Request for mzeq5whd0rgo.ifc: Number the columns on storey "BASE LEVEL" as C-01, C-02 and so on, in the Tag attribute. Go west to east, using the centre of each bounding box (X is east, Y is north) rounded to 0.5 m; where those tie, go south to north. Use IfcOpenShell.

First a look at what the model holds.

```python
import ifcopenshell
import ifcopenshell.util.element
import ifcopenshell.util.placement

model = ifcopenshell.open("mzeq5whd0rgo.ifc")
print(model.schema)
storey = next(s for s in model.by_type("IfcBuildingStorey") if s.Name == "BASE LEVEL")
columns = [e for e in ifcopenshell.util.element.get_decomposition(storey) if e.is_a("IfcColumn")]
for e in sorted(columns, key=lambda e: e.id()):
    origin = ifcopenshell.util.placement.get_local_placement(e.ObjectPlacement)[:3, 3]
    print(e.id(), e.Tag, e.Name, origin.round(2) + 0.0, sep=" | ")
```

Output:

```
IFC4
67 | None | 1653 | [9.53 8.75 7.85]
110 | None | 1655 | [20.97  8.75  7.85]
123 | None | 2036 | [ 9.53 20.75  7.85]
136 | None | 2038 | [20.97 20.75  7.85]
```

```python
import ifcopenshell
import ifcopenshell.geom
import ifcopenshell.util.element
import ifcopenshell.util.shape

model = ifcopenshell.open("mzeq5whd0rgo.ifc")
settings = ifcopenshell.geom.settings()
settings.set("use-world-coords", True)


def centre(element):
    shape = ifcopenshell.geom.create_shape(settings, element)
    return ifcopenshell.util.shape.get_bbox_centroid(shape.geometry)


storey = next(s for s in model.by_type("IfcBuildingStorey") if s.Name == "BASE LEVEL")
columns = [e for e in ifcopenshell.util.element.get_decomposition(storey) if e.is_a("IfcColumn")]

# Insertion points can sit at a corner or the storey origin, so sort by the geometry (in metres).
centres = {e: centre(e) for e in columns}
columns.sort(key=lambda e: (round(centres[e][0] / 0.5), centres[e][1]))

for i, e in enumerate(columns, start=1):
    number = f"C-{i:02d}"
    e.Tag = number
    print(e.id(), number)

model.write("mzeq5whd0rgo_v2.ifc")
```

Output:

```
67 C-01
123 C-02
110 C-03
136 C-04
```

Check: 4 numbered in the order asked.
